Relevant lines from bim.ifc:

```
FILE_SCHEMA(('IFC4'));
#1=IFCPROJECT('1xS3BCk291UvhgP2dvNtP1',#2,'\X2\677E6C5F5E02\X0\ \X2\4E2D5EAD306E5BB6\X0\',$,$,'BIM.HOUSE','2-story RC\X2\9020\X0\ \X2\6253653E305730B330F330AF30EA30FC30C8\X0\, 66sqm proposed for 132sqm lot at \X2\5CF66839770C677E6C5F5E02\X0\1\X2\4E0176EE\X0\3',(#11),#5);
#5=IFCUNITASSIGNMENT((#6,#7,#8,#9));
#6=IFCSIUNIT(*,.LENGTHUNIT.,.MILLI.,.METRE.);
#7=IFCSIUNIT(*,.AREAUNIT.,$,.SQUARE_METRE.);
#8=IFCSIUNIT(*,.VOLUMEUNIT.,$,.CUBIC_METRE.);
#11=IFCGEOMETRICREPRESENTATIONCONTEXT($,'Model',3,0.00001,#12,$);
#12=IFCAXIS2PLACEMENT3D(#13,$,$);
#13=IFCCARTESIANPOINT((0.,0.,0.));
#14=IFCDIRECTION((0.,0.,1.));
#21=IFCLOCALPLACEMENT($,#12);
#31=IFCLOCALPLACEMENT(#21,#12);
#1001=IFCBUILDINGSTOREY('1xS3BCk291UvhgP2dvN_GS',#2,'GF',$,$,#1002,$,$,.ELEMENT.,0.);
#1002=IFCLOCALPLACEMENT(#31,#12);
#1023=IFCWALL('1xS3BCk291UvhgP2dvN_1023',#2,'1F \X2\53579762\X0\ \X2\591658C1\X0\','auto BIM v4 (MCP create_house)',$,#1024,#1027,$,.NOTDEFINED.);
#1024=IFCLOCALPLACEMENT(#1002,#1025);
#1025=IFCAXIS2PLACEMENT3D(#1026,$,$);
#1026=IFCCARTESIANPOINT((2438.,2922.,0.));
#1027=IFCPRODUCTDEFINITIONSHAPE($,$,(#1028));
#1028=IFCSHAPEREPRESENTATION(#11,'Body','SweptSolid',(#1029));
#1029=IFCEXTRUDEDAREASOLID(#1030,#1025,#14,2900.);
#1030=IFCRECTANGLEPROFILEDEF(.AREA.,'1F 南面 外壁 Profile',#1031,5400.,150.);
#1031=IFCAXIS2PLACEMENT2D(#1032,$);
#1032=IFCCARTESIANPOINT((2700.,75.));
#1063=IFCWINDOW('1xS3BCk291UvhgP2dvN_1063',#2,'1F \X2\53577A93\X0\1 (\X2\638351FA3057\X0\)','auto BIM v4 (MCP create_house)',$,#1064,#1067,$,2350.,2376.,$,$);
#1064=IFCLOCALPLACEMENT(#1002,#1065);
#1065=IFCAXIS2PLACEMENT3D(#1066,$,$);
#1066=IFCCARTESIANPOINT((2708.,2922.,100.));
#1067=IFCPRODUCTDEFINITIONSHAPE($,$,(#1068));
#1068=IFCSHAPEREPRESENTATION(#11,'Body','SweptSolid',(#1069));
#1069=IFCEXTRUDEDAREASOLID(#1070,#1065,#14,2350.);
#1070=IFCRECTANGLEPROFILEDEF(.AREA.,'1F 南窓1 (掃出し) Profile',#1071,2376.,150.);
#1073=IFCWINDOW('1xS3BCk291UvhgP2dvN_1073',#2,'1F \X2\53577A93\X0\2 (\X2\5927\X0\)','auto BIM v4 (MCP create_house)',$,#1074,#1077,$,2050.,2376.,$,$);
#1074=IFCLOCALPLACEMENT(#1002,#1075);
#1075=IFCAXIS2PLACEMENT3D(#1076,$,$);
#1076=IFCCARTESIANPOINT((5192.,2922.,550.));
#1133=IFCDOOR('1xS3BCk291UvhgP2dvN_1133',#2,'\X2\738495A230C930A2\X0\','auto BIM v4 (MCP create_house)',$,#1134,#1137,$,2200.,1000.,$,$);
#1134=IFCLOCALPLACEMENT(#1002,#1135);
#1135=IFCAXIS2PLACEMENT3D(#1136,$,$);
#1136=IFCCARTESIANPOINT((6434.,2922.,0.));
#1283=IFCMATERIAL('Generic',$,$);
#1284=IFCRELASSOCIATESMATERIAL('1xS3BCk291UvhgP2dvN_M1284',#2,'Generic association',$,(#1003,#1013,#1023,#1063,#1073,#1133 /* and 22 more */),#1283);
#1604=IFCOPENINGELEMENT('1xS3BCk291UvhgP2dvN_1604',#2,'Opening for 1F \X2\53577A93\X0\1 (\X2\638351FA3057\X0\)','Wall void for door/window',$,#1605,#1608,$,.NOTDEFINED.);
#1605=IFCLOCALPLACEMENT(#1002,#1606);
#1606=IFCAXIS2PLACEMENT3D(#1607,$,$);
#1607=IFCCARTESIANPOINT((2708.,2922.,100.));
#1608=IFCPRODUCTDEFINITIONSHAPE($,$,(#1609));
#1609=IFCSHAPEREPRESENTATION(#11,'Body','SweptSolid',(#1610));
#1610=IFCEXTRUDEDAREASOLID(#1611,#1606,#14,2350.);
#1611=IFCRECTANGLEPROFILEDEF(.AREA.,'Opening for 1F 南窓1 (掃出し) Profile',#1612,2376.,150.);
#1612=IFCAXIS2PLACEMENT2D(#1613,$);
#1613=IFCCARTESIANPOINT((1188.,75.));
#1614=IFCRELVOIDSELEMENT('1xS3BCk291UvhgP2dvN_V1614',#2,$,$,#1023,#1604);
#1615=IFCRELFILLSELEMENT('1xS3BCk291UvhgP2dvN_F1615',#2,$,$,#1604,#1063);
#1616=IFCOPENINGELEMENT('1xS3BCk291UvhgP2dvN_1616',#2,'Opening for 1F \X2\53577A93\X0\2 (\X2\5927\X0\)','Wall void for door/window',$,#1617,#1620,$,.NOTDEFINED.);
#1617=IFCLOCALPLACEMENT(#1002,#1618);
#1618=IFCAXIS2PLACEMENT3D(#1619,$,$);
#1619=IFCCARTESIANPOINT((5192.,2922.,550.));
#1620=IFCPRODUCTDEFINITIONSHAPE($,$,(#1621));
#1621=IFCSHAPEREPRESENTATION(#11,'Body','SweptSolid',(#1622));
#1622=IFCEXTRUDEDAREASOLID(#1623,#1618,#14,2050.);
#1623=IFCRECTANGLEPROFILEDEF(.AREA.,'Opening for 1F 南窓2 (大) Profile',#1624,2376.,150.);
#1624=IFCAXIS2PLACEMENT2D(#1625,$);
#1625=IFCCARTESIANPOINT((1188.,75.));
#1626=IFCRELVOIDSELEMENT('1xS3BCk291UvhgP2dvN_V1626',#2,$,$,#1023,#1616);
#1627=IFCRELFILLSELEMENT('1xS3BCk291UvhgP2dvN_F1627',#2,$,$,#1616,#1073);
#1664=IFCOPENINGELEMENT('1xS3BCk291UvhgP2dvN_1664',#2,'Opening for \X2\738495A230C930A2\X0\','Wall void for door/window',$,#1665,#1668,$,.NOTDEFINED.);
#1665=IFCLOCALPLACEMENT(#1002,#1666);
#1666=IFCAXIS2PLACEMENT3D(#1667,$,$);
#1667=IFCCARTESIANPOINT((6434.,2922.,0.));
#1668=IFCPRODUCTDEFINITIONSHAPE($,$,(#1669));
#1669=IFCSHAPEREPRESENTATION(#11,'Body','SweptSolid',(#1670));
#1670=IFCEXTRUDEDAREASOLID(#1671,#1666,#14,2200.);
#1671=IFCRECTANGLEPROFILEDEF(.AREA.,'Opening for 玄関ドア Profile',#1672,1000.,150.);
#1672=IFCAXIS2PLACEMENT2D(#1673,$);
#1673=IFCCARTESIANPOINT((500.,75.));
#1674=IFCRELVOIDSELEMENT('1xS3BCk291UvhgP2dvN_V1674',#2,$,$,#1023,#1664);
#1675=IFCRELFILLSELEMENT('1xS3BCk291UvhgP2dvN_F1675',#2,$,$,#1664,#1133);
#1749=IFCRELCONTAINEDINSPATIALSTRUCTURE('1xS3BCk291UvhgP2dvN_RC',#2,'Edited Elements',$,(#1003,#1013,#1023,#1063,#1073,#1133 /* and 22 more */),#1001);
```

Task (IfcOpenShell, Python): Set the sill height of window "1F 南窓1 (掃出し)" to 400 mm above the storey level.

```python
import numpy as np
import ifcopenshell
import ifcopenshell.api.geometry
import ifcopenshell.geom
import ifcopenshell.util.element
import ifcopenshell.util.placement
import ifcopenshell.util.shape
import ifcopenshell.util.unit

model = ifcopenshell.open("bim.ifc")
unit_scale = ifcopenshell.util.unit.calculate_unit_scale(model)

window = model.by_guid("1xS3BCk291UvhgP2dvN_1063")
opening = window.FillsVoids[0].RelatingOpeningElement
storey = ifcopenshell.util.element.get_container(window, ifc_class="IfcBuildingStorey")
level = ifcopenshell.util.placement.get_local_placement(storey.ObjectPlacement)[2, 3]

# The opening's origin need not be at the sill, so measure its lowest point.
shape = ifcopenshell.geom.create_shape(ifcopenshell.geom.settings(), opening)
bottom = ifcopenshell.util.shape.get_shape_bottom_elevation(shape, shape.geometry) / unit_scale
dz = level + 0.4 / unit_scale - bottom

shift = np.array([0.0, 0.0, dz])
# The window is not placed relative to its opening, so move both.
for product in (opening, window):
    matrix = ifcopenshell.util.placement.get_local_placement(product.ObjectPlacement)
    matrix[:3, 3] += shift
    ifcopenshell.api.geometry.edit_object_placement(model, product=product, matrix=matrix, is_si=False)

print(f"moved by {dz * unit_scale:+.3f} m")

model.write("bim_rev.ifc")
```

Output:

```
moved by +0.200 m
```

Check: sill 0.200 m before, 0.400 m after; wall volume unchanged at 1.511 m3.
